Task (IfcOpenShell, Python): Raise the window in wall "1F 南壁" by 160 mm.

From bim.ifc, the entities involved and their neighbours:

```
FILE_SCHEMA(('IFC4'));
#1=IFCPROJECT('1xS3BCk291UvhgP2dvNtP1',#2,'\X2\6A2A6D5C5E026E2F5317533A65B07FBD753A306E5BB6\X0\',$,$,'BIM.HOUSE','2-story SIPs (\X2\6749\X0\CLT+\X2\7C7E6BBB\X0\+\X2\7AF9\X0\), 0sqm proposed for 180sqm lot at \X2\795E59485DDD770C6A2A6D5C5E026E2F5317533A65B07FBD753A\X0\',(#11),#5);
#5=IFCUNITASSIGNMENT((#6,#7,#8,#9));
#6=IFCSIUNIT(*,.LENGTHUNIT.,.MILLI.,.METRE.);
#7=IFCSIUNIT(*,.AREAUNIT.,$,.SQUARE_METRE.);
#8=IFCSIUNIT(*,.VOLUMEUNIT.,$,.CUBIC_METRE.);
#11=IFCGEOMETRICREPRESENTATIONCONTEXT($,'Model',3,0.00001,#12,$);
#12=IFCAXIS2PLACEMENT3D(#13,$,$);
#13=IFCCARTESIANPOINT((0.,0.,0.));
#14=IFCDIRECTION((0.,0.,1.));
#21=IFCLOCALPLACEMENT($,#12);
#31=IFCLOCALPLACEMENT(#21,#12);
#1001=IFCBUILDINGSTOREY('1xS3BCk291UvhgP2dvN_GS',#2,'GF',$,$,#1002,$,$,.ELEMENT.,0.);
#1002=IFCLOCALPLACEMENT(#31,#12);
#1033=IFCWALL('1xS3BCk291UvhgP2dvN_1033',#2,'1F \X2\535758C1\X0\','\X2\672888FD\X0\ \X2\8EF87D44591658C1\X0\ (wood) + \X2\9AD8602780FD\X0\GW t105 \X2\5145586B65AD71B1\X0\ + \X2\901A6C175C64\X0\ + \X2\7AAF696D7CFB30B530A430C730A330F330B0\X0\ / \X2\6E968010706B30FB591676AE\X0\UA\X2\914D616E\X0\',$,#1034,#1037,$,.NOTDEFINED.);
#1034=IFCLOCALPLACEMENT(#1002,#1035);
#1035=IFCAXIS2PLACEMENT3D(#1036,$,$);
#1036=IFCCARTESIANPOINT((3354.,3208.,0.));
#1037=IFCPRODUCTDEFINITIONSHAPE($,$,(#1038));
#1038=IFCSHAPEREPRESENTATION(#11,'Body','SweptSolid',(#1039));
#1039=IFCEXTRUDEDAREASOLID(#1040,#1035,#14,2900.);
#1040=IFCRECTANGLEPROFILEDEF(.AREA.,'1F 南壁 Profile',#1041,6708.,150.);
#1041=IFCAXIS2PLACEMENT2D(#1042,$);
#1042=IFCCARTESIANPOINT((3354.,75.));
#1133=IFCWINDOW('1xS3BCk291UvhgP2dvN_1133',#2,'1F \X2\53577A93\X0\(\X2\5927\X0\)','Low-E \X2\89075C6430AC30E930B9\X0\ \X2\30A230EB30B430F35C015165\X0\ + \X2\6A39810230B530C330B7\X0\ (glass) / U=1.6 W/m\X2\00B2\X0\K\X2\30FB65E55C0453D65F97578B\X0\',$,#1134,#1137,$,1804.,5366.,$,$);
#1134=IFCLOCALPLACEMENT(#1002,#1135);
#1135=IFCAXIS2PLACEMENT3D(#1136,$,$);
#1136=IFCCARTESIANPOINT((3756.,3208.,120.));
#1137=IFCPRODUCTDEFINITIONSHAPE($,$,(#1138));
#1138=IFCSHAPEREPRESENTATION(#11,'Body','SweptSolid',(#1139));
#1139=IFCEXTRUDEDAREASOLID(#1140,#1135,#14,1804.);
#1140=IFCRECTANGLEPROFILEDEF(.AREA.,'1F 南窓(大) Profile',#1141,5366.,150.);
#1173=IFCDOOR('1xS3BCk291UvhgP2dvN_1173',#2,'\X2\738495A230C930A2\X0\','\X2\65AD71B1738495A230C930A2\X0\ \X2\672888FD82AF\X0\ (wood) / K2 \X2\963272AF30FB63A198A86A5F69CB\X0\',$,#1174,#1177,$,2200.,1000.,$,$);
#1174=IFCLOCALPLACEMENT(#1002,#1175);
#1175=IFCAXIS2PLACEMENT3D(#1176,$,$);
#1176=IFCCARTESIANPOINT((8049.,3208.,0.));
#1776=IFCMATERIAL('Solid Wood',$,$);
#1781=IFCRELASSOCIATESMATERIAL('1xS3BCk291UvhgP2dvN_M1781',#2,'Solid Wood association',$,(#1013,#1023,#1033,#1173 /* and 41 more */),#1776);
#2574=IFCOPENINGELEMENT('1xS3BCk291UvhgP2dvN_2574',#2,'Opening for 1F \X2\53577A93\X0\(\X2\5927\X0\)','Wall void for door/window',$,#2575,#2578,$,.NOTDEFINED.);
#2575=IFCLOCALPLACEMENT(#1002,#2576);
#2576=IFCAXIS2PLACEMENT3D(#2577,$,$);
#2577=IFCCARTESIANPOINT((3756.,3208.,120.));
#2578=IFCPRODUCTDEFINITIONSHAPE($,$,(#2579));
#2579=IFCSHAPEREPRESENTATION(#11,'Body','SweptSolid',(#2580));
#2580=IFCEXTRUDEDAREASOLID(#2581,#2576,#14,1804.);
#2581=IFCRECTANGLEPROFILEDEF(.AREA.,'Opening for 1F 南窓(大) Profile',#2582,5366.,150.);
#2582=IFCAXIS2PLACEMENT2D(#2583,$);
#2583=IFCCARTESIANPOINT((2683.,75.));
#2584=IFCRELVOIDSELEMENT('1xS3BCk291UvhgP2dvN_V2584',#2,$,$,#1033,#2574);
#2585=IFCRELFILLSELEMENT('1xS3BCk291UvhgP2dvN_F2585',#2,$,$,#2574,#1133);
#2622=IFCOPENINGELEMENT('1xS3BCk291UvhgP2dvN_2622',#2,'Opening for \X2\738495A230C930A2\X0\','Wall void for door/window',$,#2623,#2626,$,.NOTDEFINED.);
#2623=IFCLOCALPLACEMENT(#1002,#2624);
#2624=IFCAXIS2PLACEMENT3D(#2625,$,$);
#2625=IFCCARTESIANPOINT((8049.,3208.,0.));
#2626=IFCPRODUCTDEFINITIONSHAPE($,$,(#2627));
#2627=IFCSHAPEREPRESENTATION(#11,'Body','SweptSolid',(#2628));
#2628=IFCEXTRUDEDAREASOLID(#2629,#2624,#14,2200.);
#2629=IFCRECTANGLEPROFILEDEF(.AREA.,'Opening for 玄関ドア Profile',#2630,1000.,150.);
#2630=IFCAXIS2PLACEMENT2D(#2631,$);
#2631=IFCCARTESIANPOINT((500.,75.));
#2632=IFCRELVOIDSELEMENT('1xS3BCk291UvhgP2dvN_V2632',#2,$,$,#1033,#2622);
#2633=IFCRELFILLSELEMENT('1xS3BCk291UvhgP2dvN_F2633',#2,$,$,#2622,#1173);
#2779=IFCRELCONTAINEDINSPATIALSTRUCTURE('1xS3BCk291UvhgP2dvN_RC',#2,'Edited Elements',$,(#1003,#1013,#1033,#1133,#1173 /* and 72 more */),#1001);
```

```python
import numpy as np
import ifcopenshell
import ifcopenshell.api.geometry
import ifcopenshell.util.placement
import ifcopenshell.util.unit

model = ifcopenshell.open("bim.ifc")
unit_scale = ifcopenshell.util.unit.calculate_unit_scale(model)

window = model.by_id(1133)
opening = window.FillsVoids[0].RelatingOpeningElement
dz = 0.16 / unit_scale

shift = np.array([0.0, 0.0, dz])
# The window is not placed relative to its opening, so move both.
for product in (opening, window):
    matrix = ifcopenshell.util.placement.get_local_placement(product.ObjectPlacement)
    matrix[:3, 3] += shift
    ifcopenshell.api.geometry.edit_object_placement(model, product=product, matrix=matrix, is_si=False)

print(f"moved by {dz * unit_scale:+.3f} m")

model.write("bim_v2.ifc")
```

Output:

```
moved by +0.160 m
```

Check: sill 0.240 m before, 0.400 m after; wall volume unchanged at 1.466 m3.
